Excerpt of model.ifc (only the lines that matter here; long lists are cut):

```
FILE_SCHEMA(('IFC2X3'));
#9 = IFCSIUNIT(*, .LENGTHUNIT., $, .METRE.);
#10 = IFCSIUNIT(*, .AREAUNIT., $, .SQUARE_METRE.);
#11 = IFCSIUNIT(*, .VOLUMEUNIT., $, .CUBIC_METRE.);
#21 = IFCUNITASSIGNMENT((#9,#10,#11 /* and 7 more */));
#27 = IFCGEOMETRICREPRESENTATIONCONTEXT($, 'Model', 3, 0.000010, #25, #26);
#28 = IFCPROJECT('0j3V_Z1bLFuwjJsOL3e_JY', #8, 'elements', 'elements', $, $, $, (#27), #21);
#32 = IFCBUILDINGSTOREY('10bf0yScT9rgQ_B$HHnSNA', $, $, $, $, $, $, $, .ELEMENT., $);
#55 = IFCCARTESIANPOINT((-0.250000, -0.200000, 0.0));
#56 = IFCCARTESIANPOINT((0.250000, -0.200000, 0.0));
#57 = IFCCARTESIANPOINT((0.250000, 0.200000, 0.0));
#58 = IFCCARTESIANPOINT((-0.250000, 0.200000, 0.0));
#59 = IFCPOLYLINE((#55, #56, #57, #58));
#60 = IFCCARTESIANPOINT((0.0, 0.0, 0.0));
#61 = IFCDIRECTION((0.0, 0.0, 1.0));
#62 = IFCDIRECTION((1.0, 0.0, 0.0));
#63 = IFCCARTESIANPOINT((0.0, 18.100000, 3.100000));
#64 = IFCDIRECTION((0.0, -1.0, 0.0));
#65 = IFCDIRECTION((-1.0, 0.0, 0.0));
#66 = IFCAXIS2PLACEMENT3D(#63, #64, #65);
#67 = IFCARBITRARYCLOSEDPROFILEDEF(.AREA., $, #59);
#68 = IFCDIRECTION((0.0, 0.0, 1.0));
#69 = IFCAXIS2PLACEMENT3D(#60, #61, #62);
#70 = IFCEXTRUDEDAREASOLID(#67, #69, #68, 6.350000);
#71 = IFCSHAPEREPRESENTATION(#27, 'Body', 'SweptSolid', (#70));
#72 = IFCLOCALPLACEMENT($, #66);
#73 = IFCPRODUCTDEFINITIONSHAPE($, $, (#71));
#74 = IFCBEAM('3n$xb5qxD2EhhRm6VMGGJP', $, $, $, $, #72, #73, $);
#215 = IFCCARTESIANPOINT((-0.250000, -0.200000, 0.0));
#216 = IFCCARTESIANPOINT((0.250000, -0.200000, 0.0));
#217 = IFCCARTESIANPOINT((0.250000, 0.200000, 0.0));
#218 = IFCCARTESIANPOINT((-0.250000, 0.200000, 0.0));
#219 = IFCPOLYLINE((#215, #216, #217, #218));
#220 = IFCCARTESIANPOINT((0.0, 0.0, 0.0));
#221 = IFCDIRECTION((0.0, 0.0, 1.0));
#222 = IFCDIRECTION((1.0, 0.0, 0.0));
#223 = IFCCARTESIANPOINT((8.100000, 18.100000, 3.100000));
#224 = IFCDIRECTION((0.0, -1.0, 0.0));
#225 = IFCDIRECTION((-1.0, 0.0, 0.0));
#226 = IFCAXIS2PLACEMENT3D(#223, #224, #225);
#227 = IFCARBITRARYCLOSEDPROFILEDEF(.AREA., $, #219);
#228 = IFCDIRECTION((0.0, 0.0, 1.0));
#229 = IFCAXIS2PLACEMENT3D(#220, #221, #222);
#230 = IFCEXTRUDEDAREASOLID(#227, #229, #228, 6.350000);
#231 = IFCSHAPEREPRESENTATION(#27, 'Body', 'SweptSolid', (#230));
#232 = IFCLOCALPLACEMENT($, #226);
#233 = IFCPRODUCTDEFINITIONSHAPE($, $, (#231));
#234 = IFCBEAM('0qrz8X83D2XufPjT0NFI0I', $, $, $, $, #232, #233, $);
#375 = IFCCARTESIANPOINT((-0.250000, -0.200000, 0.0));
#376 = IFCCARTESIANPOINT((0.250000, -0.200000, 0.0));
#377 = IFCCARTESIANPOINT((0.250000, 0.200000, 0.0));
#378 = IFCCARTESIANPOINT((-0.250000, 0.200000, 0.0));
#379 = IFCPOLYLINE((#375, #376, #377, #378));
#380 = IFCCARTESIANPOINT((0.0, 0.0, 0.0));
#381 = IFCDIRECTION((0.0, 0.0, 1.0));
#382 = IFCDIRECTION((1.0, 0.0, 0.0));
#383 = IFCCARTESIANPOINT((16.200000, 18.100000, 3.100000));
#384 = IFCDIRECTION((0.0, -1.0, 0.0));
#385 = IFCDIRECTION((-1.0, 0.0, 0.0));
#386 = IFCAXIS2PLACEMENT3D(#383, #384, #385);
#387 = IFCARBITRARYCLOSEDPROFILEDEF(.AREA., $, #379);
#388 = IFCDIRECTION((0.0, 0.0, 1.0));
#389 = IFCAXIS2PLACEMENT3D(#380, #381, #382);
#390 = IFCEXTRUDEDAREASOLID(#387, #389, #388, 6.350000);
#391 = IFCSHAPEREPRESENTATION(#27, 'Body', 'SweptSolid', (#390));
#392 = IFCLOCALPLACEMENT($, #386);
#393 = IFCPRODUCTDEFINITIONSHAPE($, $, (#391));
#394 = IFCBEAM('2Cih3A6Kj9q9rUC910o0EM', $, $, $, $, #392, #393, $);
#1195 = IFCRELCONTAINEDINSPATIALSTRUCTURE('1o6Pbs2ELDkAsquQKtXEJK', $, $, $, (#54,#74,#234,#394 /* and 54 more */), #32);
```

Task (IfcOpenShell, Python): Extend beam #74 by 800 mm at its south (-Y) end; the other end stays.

```python
import ifcopenshell
import ifcopenshell.util.unit

model = ifcopenshell.open("model.ifc")
unit_scale = ifcopenshell.util.unit.calculate_unit_scale(model)

member = model.by_id(74)
change = 0.8 / unit_scale

# The extrusion runs towards the end named, so only its depth changes.
body = next(r for r in member.Representation.Representations if r.RepresentationIdentifier == "Body")
solid = body.Items[0]
old_length = solid.Depth
solid.Depth += change

print(f"length {old_length:g} -> {solid.Depth:g}")

model.write("model_updated.ifc")
```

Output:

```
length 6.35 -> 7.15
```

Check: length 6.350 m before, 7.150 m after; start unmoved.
